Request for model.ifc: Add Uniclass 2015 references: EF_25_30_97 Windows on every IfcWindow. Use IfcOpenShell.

First a look at what the model holds.

```python
import ifcopenshell

model = ifcopenshell.open("model.ifc")
print(model.schema)
print("classifications:", [c.Name for c in model.by_type("IfcClassification")])
for ifc_class in ("IfcDoor", "IfcRoof", "IfcStair", "IfcWall", "IfcWindow"):
    print(ifc_class, len(model.by_type(ifc_class)))
```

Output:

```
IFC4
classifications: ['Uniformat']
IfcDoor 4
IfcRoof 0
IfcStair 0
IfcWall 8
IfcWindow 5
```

```python
import ifcopenshell
import ifcopenshell.api.classification

model = ifcopenshell.open("model.ifc")

system = ifcopenshell.api.classification.add_classification(model, classification="Uniclass 2015")

codes = {
    "IfcWindow": ("EF_25_30_97", "Windows"),
}
for ifc_class, (code, name) in codes.items():
    products = model.by_type(ifc_class)
    ifcopenshell.api.classification.add_reference(
        model, products=products, classification=system, identification=code, name=name
    )
    print(code, len(products))

model.write("model_rev.ifc")
```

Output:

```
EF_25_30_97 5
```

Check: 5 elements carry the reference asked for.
